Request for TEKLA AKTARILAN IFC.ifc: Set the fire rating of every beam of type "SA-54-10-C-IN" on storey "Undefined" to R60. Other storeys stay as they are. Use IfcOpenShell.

First a look at what the model holds.

```python
import ifcopenshell
import ifcopenshell.util.element

model = ifcopenshell.open("TEKLA AKTARILAN IFC.ifc")
print(model.schema)
storey = next(s for s in model.by_type("IfcBuildingStorey") if s.Name == "Undefined")
beams = [e for e in ifcopenshell.util.element.get_decomposition(storey) if e.is_a("IfcBeam")]
seen = {}
for e in beams:
    element_type = ifcopenshell.util.element.get_type(e)
    key = (element_type.Name if element_type != e and element_type else None, ifcopenshell.util.element.get_pset(e, "Pset_BeamCommon", "FireRating"))
    seen[key] = seen.get(key, 0) + 1
for (name, value), count in sorted(seen.items(), key=str):
    print(count, "x", name, "|", value)
```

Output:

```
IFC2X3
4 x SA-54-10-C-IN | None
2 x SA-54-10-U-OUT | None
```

```python
import ifcopenshell
import ifcopenshell.api.pset
import ifcopenshell.util.element

model = ifcopenshell.open("TEKLA AKTARILAN IFC.ifc")

storey = next(s for s in model.by_type("IfcBuildingStorey") if s.Name == "Undefined")
beams = [e for e in ifcopenshell.util.element.get_decomposition(storey) if e.is_a("IfcBeam")]

count = 0
for e in beams:
    element_type = ifcopenshell.util.element.get_type(e)
    if element_type in (None, e) or element_type.Name != "SA-54-10-C-IN":
        continue
    # add_pset returns the element's existing set when there is one.
    pset = ifcopenshell.api.pset.add_pset(model, product=e, name="Pset_BeamCommon")
    ifcopenshell.api.pset.edit_pset(model, pset=pset, properties={"FireRating": "R60"})
    count += 1

print(count, "beams updated")

model.write("TEKLA AKTARILAN IFC_rev.ifc")
```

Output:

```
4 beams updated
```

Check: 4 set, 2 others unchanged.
